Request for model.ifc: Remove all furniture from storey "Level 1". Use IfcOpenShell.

First a look at what the model holds.

```python
import ifcopenshell
import ifcopenshell.util.element

model = ifcopenshell.open("model.ifc")
print(model.schema)
storey = next(s for s in model.by_type("IfcBuildingStorey") if s.Name == "Level 1")
furniture = [e for e in ifcopenshell.util.element.get_decomposition(storey) if e.is_a("IfcFurnishingElement")]
seen = {}
for e in furniture:
    element_type = ifcopenshell.util.element.get_type(e)
    name = element_type.Name if element_type not in (None, e) else None
    seen[name] = seen.get(name, 0) + 1
for name, count in sorted(seen.items(), key=str):
    print(count, "x", name)
```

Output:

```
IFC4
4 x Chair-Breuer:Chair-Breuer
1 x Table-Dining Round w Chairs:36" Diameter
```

```python
import ifcopenshell
import ifcopenshell.api.root
import ifcopenshell.util.element

model = ifcopenshell.open("model.ifc")

storey = next(s for s in model.by_type("IfcBuildingStorey") if s.Name == "Level 1")
furniture = [e for e in ifcopenshell.util.element.get_decomposition(storey) if e.is_a("IfcFurnishingElement")]

for e in furniture:
    ifcopenshell.api.root.remove_product(model, product=e)
print(len(furniture), "removed")

model.write("model-out.ifc")
```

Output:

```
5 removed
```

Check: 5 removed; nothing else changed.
